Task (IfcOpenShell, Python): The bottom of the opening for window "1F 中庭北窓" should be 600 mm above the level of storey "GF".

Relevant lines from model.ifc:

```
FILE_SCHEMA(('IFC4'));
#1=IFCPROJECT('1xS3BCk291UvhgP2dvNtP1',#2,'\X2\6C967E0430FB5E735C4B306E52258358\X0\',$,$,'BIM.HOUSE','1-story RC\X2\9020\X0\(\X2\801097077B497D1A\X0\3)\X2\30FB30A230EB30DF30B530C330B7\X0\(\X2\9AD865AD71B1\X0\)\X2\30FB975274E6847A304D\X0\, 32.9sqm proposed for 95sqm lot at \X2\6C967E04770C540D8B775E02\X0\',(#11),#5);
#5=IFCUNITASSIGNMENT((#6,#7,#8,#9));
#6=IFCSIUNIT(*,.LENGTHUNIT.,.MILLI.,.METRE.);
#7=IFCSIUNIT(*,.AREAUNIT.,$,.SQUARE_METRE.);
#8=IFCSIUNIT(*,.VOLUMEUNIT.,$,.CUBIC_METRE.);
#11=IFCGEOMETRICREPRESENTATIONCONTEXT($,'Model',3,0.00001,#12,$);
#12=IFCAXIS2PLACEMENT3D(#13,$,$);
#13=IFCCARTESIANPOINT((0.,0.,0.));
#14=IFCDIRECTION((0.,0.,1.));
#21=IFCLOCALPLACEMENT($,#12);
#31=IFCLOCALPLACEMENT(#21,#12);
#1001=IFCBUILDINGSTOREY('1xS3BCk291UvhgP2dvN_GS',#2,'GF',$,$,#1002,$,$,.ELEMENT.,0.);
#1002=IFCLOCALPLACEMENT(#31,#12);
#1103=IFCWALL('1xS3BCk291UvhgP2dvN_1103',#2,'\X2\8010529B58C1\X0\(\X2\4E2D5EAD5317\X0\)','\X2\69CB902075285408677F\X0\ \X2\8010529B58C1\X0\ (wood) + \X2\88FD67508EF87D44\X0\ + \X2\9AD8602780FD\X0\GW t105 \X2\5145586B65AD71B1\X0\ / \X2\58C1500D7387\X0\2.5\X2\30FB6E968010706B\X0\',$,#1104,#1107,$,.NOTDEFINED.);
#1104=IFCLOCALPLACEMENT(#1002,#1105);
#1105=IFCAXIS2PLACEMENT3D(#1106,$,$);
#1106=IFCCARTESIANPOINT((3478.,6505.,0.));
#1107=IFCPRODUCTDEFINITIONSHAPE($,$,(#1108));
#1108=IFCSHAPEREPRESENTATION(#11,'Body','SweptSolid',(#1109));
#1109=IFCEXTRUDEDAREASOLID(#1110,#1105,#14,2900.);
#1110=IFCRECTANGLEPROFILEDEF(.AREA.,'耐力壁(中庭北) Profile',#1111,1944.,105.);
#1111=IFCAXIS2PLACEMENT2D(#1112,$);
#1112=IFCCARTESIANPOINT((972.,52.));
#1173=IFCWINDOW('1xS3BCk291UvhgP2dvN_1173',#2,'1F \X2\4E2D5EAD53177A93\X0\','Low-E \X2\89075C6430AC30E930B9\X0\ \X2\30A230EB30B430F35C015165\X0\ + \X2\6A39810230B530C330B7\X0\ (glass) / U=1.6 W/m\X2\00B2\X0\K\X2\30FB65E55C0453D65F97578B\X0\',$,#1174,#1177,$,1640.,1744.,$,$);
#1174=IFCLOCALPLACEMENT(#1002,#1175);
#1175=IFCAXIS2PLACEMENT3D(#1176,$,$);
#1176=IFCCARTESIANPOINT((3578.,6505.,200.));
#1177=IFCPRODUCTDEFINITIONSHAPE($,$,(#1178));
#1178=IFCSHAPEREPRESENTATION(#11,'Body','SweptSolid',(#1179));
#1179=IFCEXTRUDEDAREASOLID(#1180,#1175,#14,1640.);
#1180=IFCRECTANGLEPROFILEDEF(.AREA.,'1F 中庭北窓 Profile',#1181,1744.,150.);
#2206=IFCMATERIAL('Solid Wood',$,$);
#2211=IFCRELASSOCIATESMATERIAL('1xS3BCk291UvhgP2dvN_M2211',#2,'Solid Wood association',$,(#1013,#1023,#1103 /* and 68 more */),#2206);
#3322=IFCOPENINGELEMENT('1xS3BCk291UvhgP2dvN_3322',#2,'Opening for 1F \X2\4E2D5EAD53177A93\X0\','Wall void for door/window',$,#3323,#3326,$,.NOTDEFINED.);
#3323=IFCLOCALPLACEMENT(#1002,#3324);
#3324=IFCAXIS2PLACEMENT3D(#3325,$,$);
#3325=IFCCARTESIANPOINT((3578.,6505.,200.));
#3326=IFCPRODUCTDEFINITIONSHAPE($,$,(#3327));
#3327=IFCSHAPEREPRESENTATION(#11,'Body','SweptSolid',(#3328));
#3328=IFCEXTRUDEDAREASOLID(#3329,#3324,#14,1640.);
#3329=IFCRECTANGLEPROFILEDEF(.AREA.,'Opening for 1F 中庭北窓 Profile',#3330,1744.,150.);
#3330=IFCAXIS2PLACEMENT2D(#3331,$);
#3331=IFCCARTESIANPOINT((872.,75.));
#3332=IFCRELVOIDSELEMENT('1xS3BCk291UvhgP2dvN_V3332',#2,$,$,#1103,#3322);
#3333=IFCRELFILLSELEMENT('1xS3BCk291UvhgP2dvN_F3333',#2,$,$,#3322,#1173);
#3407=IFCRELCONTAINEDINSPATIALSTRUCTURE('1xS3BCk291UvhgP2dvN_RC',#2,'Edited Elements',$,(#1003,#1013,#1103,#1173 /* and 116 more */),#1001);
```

```python
import numpy as np
import ifcopenshell
import ifcopenshell.api.geometry
import ifcopenshell.geom
import ifcopenshell.util.element
import ifcopenshell.util.placement
import ifcopenshell.util.shape
import ifcopenshell.util.unit

model = ifcopenshell.open("model.ifc")
unit_scale = ifcopenshell.util.unit.calculate_unit_scale(model)

window = model.by_id(1173)
opening = window.FillsVoids[0].RelatingOpeningElement
storey = ifcopenshell.util.element.get_container(window, ifc_class="IfcBuildingStorey")
level = ifcopenshell.util.placement.get_local_placement(storey.ObjectPlacement)[2, 3]

# The opening's origin need not be at the sill, so measure its lowest point.
shape = ifcopenshell.geom.create_shape(ifcopenshell.geom.settings(), opening)
bottom = ifcopenshell.util.shape.get_shape_bottom_elevation(shape, shape.geometry) / unit_scale
dz = level + 600.0 - bottom

shift = np.array([0.0, 0.0, dz])
# The window is not placed relative to its opening, so move both.
for product in (opening, window):
    matrix = ifcopenshell.util.placement.get_local_placement(product.ObjectPlacement)
    matrix[:3, 3] += shift
    ifcopenshell.api.geometry.edit_object_placement(model, product=product, matrix=matrix, is_si=False)

print(f"moved by {dz * unit_scale:+.3f} m")

model.write("model-out.ifc")
```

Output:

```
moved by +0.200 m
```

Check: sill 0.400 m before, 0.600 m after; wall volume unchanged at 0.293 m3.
